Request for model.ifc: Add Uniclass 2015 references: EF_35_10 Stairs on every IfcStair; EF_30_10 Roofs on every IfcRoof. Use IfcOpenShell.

First a look at what the model holds.

```python
import ifcopenshell

model = ifcopenshell.open("model.ifc")
print(model.schema)
print("classifications:", [c.Name for c in model.by_type("IfcClassification")])
for ifc_class in ("IfcDoor", "IfcRoof", "IfcStair", "IfcWall", "IfcWindow"):
    print(ifc_class, len(model.by_type(ifc_class)))
```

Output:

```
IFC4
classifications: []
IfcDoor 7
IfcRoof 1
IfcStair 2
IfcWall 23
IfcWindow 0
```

```python
import ifcopenshell
import ifcopenshell.api.classification

model = ifcopenshell.open("model.ifc")

system = ifcopenshell.api.classification.add_classification(model, classification="Uniclass 2015")

codes = {
    "IfcStair": ("EF_35_10", "Stairs"),
    "IfcRoof": ("EF_30_10", "Roofs"),
}
for ifc_class, (code, name) in codes.items():
    products = model.by_type(ifc_class)
    ifcopenshell.api.classification.add_reference(
        model, products=products, classification=system, identification=code, name=name
    )
    print(code, len(products))

model.write("model_v2.ifc")
```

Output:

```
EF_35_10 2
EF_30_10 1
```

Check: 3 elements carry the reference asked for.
